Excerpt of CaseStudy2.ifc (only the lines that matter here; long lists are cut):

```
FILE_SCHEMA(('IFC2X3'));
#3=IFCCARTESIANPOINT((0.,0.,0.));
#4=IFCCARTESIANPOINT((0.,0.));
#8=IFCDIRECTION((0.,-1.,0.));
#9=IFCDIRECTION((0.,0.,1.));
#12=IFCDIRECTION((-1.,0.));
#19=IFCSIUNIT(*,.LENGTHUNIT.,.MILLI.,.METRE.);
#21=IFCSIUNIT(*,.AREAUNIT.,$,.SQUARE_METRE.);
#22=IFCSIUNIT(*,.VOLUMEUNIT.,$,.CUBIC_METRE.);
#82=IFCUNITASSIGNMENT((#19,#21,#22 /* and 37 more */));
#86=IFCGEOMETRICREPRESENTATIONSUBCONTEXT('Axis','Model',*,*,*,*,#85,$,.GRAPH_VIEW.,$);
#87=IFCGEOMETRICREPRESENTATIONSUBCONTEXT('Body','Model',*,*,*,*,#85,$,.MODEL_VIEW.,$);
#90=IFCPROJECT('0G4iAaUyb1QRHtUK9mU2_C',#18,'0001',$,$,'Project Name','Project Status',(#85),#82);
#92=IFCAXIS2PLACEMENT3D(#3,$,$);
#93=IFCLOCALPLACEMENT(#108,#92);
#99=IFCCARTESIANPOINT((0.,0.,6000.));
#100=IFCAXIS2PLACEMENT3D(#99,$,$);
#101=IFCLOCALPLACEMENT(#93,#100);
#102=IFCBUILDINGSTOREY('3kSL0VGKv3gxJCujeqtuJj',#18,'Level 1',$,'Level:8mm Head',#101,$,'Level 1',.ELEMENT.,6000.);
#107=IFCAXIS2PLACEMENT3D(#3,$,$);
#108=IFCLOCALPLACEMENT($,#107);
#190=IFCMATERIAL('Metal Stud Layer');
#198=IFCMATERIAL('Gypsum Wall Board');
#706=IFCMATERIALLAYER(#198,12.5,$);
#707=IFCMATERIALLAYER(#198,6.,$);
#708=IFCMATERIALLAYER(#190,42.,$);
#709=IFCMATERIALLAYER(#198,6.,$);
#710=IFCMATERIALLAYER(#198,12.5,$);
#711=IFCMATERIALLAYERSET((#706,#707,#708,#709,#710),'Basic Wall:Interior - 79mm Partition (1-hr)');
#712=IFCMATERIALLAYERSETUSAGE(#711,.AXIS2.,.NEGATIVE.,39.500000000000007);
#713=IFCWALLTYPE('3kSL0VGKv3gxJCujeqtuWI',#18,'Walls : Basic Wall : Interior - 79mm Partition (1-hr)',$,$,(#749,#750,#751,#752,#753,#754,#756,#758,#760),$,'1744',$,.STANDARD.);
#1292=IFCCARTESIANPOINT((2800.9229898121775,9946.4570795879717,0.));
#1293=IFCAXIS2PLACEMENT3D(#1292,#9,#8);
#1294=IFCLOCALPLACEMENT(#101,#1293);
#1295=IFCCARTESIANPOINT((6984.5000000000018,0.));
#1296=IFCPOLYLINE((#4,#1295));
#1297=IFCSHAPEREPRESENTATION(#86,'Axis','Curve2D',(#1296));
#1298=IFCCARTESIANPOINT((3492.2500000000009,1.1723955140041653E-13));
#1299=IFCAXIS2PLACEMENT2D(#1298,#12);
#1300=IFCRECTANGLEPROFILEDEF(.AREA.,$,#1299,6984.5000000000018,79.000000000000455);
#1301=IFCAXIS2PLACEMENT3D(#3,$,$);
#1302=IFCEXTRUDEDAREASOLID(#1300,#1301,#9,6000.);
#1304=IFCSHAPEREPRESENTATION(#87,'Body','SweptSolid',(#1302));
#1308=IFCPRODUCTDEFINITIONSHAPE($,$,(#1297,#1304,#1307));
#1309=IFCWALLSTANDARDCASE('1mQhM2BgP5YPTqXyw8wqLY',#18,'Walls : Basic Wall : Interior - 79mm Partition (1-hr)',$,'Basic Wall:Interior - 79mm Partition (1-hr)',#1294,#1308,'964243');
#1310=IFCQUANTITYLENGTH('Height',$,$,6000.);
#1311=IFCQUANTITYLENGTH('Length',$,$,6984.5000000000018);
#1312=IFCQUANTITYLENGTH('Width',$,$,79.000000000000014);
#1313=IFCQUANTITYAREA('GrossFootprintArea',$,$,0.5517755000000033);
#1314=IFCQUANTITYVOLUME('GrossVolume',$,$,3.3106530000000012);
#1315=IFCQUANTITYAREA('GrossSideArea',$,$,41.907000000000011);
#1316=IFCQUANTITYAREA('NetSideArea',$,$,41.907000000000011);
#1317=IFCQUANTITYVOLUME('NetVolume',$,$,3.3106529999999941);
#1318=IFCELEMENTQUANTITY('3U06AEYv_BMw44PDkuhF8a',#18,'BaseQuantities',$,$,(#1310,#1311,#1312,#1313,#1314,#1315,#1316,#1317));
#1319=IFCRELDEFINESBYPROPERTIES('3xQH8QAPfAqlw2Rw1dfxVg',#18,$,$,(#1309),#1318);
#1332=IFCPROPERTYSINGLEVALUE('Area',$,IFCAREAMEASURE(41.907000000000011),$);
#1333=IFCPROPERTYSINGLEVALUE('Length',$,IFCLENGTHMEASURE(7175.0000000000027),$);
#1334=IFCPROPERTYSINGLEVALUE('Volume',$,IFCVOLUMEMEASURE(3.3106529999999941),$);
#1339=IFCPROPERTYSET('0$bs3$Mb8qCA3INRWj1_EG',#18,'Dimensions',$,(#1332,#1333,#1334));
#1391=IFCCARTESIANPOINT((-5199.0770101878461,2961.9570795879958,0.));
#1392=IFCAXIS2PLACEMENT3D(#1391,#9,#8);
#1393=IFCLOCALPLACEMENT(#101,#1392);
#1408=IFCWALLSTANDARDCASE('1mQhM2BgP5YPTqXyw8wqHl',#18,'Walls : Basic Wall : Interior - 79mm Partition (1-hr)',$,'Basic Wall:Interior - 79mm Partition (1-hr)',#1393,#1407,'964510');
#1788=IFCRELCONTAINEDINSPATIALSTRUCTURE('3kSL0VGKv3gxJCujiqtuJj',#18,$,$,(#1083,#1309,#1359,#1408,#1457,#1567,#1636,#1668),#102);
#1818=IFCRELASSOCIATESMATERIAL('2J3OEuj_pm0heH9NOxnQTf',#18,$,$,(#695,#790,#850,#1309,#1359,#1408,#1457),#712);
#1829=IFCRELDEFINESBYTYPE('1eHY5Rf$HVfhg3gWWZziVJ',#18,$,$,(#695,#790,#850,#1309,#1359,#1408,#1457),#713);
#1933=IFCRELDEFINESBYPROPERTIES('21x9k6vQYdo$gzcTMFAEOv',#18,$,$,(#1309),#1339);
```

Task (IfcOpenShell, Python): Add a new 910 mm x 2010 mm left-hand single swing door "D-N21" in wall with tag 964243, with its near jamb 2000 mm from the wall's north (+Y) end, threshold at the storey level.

```python
import numpy as np
import ifcopenshell
import ifcopenshell.api.feature
import ifcopenshell.api.geometry
import ifcopenshell.api.pset
import ifcopenshell.api.root
import ifcopenshell.api.spatial
import ifcopenshell.api.type
import ifcopenshell.geom
import ifcopenshell.util.element
import ifcopenshell.util.placement
import ifcopenshell.util.representation
import ifcopenshell.util.shape
import ifcopenshell.util.unit

model = ifcopenshell.open("CaseStudy2.ifc")
unit_scale = ifcopenshell.util.unit.calculate_unit_scale(model)
area_scale = ifcopenshell.util.unit.calculate_unit_scale(model, "AREAUNIT")
volume_scale = ifcopenshell.util.unit.calculate_unit_scale(model, "VOLUMEUNIT")
settings = ifcopenshell.geom.settings()


def volume(element):
    """Net volume in cubic metres, openings subtracted."""
    shape = ifcopenshell.geom.create_shape(settings, element)
    return ifcopenshell.util.shape.get_volume(shape.geometry)


wall = model.by_id(1309)
storey = ifcopenshell.util.element.get_container(wall, ifc_class="IfcBuildingStorey")
context = ifcopenshell.util.representation.get_context(model, "Model", "Body", "MODEL_VIEW")
before = volume(wall)

width, height, from_end, sill = 0.91, 2.01, 2, 0.0  # metres

# The wall runs along its own X axis, and the end named is its -X end.
wall_shape = ifcopenshell.geom.create_shape(settings, wall)
x, y, z = ifcopenshell.util.shape.get_vertices(wall_shape.geometry).T
start = x.min() + from_end
face, thickness = float(y.min()), float(y.max() - y.min())
wall_matrix = ifcopenshell.util.placement.get_local_placement(wall.ObjectPlacement)
level = ifcopenshell.util.placement.get_local_placement(storey.ObjectPlacement)[2, 3]


def in_wall(x, y):
    """Placement at x, y metres in the wall's axes, at sill height."""
    matrix = wall_matrix.copy()
    matrix[:, 3] = wall_matrix @ np.array([x / unit_scale, y / unit_scale, 0.0, 1.0])
    matrix[2, 3] = level + sill / unit_scale
    return matrix


# Opening: a box that overshoots both wall faces by 50 mm.
opening = ifcopenshell.api.root.create_entity(model, ifc_class="IfcOpeningElement")
box = ifcopenshell.api.geometry.add_wall_representation(
    model, context=context, length=width, height=height, thickness=thickness + 0.1
)
ifcopenshell.api.geometry.assign_representation(model, product=opening, representation=box)
ifcopenshell.api.geometry.edit_object_placement(model, product=opening, matrix=in_wall(start, face - 0.05), is_si=False)
ifcopenshell.api.feature.add_feature(model, feature=opening, element=wall)

door = ifcopenshell.api.root.create_entity(model, ifc_class="IfcDoor", name="D-N21")
door.OverallWidth, door.OverallHeight = width / unit_scale, height / unit_scale
body = ifcopenshell.api.geometry.add_door_representation(
    model,
    context=context,
    overall_width=door.OverallWidth,
    overall_height=door.OverallHeight,
    operation_type="SINGLE_SWING_LEFT",
    lining_properties={"LiningDepth": thickness / unit_scale, "ThresholdDepth": thickness / unit_scale},
)
ifcopenshell.api.geometry.assign_representation(model, product=door, representation=body)
ifcopenshell.api.spatial.assign_container(model, products=[door], relating_structure=storey)
fills = ifcopenshell.api.feature.add_filling(model, opening=opening, element=door)
fills.OwnerHistory = door.OwnerHistory  # required in IFC2X3

# IFC2X3 keeps the operation on the door style.
style = ifcopenshell.api.root.create_entity(model, ifc_class="IfcDoorStyle", name="D-N21")
style.OperationType, style.ConstructionType = "SINGLE_SWING_LEFT", "NOTDEFINED"
style.ParameterTakesPrecedence = style.Sizeable = False
ifcopenshell.api.type.assign_type(model, related_objects=[door], relating_type=style)

# The lining spans the wall, so the door starts at the wall face.
ifcopenshell.api.geometry.edit_object_placement(model, product=door, matrix=in_wall(start, face), is_si=False)

after = volume(wall)

# Update the wall's stored quantities.
qto = model.by_id(ifcopenshell.util.element.get_pset(wall, "BaseQuantities", should_inherit=False)["id"])
ifcopenshell.api.pset.edit_qto(model, qto=qto, properties={
    "NetSideArea": after / thickness / area_scale,
    "NetVolume": after / volume_scale,
})
pset = model.by_id(ifcopenshell.util.element.get_pset(wall, "Dimensions", should_inherit=False)["id"])
ifcopenshell.api.pset.edit_pset(model, pset=pset, properties={
    "Area": model.create_entity("IfcAreaMeasure", after / thickness / area_scale),
    "Volume": model.create_entity("IfcVolumeMeasure", after / volume_scale),
})

print(f"wall volume {before:.3f} -> {after:.3f} m3")

model.write("CaseStudy2-out.ifc")
```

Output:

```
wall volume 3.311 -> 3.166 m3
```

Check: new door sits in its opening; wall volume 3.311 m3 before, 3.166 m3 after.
